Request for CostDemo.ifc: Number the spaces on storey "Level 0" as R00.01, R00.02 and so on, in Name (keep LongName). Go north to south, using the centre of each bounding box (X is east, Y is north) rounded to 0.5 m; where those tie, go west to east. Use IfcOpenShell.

First a look at what the model holds.

```python
import ifcopenshell
import ifcopenshell.util.element
import ifcopenshell.util.placement

model = ifcopenshell.open("CostDemo.ifc")
print(model.schema)
storey = next(s for s in model.by_type("IfcBuildingStorey") if s.Name == "Level 0")
spaces = [e for e in ifcopenshell.util.element.get_decomposition(storey) if e.is_a("IfcSpace")]
for e in sorted(spaces, key=lambda e: e.id()):
    origin = ifcopenshell.util.placement.get_local_placement(e.ObjectPlacement)[:3, 3]
    print(e.id(), e.Name, e.LongName, origin.round(2) + 0.0, sep=" | ")
```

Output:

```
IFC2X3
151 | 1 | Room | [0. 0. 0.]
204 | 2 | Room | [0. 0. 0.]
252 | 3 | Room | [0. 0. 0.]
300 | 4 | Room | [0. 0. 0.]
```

```python
import ifcopenshell
import ifcopenshell.geom
import ifcopenshell.util.element
import ifcopenshell.util.shape

model = ifcopenshell.open("CostDemo.ifc")
settings = ifcopenshell.geom.settings()
settings.set("use-world-coords", True)


def centre(element):
    shape = ifcopenshell.geom.create_shape(settings, element)
    return ifcopenshell.util.shape.get_bbox_centroid(shape.geometry)


storey = next(s for s in model.by_type("IfcBuildingStorey") if s.Name == "Level 0")
spaces = [e for e in ifcopenshell.util.element.get_decomposition(storey) if e.is_a("IfcSpace")]

# Insertion points can sit at a corner or the storey origin, so sort by the geometry (in metres).
centres = {e: centre(e) for e in spaces}
spaces.sort(key=lambda e: (-round(centres[e][1] / 0.5), centres[e][0]))

for i, e in enumerate(spaces, start=1):
    number = f"R00.{i:02d}"
    e.Name = number
    print(e.id(), number)

model.write("CostDemo_edited.ifc")
```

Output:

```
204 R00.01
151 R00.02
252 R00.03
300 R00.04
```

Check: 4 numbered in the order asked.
